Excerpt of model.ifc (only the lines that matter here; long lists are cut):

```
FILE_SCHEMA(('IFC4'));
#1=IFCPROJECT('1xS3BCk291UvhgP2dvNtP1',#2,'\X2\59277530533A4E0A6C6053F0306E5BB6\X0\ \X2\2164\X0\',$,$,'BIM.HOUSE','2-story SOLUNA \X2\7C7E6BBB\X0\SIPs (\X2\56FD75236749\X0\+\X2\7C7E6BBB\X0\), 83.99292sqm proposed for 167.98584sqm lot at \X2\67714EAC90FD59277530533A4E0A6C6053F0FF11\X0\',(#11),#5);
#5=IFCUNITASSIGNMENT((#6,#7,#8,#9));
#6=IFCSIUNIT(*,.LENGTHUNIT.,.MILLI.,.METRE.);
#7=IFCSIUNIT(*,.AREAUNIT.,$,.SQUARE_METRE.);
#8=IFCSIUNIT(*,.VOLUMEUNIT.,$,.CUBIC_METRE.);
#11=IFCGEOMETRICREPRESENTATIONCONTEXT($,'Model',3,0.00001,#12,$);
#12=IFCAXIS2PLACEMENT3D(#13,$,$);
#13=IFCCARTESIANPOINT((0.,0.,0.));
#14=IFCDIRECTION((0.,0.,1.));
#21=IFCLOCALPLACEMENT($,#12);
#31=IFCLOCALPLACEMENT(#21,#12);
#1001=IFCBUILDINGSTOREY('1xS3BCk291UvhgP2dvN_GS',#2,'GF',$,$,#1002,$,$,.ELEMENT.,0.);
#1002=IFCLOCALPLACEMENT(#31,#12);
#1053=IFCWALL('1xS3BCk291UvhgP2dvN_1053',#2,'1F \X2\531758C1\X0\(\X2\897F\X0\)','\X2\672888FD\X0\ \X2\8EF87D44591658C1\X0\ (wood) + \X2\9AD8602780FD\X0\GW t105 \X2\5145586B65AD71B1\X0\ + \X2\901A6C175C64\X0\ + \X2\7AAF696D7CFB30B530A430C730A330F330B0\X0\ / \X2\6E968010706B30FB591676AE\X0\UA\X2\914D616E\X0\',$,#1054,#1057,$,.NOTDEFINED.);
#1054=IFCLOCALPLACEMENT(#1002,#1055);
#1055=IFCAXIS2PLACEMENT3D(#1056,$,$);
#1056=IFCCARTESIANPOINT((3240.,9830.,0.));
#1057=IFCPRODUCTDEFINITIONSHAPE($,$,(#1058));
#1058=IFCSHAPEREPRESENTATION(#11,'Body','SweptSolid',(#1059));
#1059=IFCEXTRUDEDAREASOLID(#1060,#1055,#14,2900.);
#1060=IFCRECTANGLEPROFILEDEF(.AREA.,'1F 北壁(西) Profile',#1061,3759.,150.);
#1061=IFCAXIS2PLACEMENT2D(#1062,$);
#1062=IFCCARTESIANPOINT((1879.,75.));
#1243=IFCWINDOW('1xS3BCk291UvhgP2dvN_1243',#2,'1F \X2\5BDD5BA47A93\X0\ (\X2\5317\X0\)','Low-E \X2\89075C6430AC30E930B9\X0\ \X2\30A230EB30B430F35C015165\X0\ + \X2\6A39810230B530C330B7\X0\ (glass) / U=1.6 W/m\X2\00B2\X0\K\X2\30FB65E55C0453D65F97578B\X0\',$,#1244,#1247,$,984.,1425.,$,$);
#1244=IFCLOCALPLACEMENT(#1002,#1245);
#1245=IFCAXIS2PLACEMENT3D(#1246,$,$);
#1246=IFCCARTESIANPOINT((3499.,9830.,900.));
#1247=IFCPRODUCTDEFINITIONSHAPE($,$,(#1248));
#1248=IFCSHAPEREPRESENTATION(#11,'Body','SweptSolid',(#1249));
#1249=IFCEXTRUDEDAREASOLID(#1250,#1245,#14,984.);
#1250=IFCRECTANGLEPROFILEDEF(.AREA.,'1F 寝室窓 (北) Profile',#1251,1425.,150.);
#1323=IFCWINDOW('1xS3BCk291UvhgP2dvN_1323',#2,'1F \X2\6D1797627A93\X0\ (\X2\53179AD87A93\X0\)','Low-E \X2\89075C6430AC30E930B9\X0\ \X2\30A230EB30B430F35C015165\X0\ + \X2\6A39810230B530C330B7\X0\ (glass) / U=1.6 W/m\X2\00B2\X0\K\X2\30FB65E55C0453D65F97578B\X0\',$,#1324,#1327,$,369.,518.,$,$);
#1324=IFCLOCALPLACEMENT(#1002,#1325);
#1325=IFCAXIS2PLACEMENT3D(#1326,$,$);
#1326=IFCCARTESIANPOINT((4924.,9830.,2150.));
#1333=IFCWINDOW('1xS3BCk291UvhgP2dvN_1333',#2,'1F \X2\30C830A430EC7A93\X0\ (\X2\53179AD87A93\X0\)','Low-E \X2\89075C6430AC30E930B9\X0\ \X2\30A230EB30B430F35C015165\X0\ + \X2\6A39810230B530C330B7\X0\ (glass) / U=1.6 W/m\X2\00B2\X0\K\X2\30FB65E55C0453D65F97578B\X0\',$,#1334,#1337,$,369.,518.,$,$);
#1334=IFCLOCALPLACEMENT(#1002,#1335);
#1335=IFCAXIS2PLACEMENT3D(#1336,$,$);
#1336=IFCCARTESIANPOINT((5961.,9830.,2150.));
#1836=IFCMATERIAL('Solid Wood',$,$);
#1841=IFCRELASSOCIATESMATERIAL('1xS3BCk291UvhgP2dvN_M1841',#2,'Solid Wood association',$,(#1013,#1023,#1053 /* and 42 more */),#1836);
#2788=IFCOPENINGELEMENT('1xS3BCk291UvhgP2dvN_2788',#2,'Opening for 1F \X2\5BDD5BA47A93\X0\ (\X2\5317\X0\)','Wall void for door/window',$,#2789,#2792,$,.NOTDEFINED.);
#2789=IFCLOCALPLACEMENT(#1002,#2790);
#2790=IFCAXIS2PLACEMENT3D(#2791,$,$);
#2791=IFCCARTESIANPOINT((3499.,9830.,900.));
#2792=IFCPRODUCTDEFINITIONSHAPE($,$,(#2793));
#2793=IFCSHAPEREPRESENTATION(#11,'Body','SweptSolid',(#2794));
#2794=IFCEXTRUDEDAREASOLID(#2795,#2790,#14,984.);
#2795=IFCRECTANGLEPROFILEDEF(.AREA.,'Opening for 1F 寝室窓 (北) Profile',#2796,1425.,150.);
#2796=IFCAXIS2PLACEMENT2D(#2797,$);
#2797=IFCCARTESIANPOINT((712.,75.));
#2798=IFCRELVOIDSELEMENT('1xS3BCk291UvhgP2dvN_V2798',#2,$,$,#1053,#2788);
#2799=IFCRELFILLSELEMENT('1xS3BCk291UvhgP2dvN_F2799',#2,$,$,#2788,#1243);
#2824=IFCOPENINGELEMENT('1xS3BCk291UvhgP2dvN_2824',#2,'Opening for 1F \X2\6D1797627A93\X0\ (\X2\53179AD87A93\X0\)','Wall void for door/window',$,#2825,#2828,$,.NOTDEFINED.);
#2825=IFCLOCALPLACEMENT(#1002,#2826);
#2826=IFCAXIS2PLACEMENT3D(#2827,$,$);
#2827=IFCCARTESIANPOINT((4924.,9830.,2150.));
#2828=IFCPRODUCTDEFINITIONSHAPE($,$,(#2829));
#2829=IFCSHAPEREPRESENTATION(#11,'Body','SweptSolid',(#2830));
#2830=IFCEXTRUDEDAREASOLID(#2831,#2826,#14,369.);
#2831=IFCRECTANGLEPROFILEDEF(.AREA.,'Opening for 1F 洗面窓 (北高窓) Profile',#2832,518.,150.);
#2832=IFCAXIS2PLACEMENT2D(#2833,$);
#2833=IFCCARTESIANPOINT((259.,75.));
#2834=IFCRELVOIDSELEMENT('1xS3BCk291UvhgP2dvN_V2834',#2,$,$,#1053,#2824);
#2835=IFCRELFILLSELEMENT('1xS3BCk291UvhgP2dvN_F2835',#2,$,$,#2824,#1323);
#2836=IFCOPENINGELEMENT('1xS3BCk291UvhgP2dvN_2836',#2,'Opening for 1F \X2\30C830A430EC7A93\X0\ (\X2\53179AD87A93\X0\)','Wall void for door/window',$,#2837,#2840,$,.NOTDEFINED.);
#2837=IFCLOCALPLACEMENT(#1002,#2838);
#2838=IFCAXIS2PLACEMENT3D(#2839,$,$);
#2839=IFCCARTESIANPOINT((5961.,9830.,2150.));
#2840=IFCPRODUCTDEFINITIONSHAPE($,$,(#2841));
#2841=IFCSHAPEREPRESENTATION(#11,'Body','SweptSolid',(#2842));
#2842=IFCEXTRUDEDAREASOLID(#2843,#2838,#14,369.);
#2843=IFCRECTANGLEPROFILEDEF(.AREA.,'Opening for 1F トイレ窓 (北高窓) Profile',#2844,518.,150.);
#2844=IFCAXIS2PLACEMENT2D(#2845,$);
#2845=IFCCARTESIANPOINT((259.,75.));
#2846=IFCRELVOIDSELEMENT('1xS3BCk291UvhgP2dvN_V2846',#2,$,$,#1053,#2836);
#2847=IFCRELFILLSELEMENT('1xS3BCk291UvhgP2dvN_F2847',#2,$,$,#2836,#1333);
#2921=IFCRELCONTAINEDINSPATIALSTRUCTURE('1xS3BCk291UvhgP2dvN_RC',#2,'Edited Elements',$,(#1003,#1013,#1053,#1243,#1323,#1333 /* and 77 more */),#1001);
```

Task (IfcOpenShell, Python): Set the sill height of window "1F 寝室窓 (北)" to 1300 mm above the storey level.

```python
import numpy as np
import ifcopenshell
import ifcopenshell.api.geometry
import ifcopenshell.geom
import ifcopenshell.util.element
import ifcopenshell.util.placement
import ifcopenshell.util.shape
import ifcopenshell.util.unit

model = ifcopenshell.open("model.ifc")
unit_scale = ifcopenshell.util.unit.calculate_unit_scale(model)

window = model.by_guid("1xS3BCk291UvhgP2dvN_1243")
opening = window.FillsVoids[0].RelatingOpeningElement
storey = ifcopenshell.util.element.get_container(window, ifc_class="IfcBuildingStorey")
level = ifcopenshell.util.placement.get_local_placement(storey.ObjectPlacement)[2, 3]

# The opening's origin need not be at the sill, so measure its lowest point.
shape = ifcopenshell.geom.create_shape(ifcopenshell.geom.settings(), opening)
bottom = ifcopenshell.util.shape.get_shape_bottom_elevation(shape, shape.geometry) / unit_scale
dz = level + 1300.0 - bottom

shift = np.array([0.0, 0.0, dz])
# The window is not placed relative to its opening, so move both.
for product in (opening, window):
    matrix = ifcopenshell.util.placement.get_local_placement(product.ObjectPlacement)
    matrix[:3, 3] += shift
    ifcopenshell.api.geometry.edit_object_placement(model, product=product, matrix=matrix, is_si=False)

print(f"moved by {dz * unit_scale:+.3f} m")

model.write("model_edited.ifc")
```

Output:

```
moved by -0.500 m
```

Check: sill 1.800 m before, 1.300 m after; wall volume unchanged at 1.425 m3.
